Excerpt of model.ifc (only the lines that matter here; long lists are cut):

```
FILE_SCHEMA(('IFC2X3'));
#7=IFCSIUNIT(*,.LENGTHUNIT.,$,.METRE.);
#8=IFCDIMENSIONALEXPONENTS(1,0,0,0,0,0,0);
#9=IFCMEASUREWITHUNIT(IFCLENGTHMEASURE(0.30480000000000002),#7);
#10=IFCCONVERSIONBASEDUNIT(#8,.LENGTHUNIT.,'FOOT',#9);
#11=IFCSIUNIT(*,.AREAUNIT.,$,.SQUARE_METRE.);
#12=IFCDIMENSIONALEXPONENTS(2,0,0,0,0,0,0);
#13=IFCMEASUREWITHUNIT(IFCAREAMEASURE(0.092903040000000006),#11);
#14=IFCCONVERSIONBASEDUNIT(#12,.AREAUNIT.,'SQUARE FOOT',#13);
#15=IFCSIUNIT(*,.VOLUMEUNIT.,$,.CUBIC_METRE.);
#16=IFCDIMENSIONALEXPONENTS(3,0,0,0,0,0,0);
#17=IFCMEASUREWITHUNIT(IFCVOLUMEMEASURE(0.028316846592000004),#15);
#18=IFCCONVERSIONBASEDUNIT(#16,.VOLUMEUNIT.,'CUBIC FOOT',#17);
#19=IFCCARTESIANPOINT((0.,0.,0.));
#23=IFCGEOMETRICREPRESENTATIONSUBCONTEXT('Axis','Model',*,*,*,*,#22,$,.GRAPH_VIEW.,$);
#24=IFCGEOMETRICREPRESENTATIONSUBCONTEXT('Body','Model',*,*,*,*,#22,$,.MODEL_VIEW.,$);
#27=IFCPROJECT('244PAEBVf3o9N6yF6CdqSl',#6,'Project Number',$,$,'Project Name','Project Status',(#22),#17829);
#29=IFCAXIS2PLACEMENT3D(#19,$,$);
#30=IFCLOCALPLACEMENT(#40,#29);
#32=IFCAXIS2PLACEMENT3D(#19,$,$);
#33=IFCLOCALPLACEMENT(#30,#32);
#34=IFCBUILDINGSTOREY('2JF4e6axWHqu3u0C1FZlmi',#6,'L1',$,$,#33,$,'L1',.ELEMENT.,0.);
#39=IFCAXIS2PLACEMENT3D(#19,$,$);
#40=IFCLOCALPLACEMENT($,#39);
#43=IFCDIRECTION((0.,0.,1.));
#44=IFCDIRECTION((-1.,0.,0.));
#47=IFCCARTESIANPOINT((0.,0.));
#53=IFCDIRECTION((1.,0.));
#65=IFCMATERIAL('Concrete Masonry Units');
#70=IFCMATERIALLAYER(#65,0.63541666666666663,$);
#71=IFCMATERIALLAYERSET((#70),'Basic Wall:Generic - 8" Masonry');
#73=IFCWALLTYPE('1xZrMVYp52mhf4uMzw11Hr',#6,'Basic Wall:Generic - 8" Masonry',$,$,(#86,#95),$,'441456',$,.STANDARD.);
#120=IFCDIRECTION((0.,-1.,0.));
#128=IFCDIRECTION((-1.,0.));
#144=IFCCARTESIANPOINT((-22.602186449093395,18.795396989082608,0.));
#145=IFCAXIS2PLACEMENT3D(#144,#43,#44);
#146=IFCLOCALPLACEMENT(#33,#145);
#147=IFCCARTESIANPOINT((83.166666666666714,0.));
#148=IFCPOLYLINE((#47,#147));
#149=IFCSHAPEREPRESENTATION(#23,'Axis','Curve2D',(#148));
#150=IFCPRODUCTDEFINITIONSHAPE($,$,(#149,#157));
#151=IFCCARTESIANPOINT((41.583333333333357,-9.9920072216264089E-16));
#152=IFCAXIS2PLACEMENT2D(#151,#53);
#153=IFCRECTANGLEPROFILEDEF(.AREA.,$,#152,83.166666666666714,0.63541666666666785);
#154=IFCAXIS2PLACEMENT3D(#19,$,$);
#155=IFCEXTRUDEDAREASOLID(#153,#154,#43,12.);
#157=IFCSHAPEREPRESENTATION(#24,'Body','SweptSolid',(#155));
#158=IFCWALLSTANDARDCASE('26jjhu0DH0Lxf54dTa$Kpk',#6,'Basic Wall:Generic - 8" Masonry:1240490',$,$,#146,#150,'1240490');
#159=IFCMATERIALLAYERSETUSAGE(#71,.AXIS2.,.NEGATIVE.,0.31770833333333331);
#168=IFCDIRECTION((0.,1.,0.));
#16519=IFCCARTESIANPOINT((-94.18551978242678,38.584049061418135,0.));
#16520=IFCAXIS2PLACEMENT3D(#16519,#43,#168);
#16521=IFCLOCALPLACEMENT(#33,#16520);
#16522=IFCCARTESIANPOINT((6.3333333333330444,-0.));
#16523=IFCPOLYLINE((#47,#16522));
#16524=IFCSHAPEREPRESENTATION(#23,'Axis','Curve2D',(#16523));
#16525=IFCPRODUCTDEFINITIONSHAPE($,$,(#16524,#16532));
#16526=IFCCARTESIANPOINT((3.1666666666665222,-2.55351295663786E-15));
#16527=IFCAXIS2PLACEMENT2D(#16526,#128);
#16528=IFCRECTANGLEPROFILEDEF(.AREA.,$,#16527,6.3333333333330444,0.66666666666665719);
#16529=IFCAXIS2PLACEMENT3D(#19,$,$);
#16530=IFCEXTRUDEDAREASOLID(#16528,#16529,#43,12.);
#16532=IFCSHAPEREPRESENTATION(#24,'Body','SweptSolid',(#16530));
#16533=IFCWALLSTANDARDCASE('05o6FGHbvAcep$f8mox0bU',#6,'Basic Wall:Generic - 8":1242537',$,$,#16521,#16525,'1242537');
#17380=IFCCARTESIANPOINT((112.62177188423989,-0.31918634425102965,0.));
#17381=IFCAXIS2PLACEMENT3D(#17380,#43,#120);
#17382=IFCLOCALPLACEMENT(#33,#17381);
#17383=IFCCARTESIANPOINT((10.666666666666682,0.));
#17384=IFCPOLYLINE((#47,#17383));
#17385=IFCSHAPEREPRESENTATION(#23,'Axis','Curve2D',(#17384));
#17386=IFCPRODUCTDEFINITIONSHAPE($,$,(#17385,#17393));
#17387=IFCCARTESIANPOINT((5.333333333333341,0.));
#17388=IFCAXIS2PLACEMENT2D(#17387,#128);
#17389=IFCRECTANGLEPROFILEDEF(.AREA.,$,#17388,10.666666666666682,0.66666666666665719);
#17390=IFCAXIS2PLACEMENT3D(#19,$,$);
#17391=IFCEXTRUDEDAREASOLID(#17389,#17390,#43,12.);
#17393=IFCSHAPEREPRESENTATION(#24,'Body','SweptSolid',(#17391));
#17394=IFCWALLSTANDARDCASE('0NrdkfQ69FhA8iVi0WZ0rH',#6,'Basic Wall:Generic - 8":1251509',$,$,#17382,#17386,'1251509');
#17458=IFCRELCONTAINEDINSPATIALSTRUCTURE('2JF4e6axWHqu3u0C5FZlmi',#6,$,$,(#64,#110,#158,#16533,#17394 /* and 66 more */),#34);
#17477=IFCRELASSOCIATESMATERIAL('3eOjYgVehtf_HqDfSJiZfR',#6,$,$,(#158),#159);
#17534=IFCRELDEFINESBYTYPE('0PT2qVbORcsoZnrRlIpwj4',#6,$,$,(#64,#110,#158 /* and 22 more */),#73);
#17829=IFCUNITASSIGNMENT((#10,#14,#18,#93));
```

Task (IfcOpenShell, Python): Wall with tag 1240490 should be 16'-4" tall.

```python
import ifcopenshell
import ifcopenshell.geom
import ifcopenshell.util.representation
import ifcopenshell.util.shape
import ifcopenshell.util.unit

model = ifcopenshell.open("model.ifc")
unit_scale = ifcopenshell.util.unit.calculate_unit_scale(model)
settings = ifcopenshell.geom.settings()


def volume(element):
    """Net volume in cubic metres, openings subtracted."""
    shape = ifcopenshell.geom.create_shape(settings, element)
    return ifcopenshell.util.shape.get_volume(shape.geometry)


wall = model.by_guid("26jjhu0DH0Lxf54dTa$Kpk")
before = volume(wall)

body = ifcopenshell.util.representation.get_representation(wall, "Model", "Body")
solid = body.Items[0]
old_height = solid.Depth
solid.Depth = 196 * 0.0254 / unit_scale
after = volume(wall)

print(f"height {old_height:g} -> {solid.Depth:g}, volume {before:.3f} -> {after:.3f} m3")

model.write("model_edited.ifc")
```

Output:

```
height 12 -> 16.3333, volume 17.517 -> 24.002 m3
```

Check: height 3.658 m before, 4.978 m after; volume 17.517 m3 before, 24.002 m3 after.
